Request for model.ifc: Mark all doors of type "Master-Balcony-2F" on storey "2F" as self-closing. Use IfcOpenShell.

First a look at what the model holds.

```python
import ifcopenshell
import ifcopenshell.util.element

model = ifcopenshell.open("model.ifc")
print(model.schema)
storey = next(s for s in model.by_type("IfcBuildingStorey") if s.Name == "2F")
doors = [e for e in ifcopenshell.util.element.get_decomposition(storey) if e.is_a("IfcDoor")]
seen = {}
for e in doors:
    element_type = ifcopenshell.util.element.get_type(e)
    key = (element_type.Name if element_type != e and element_type else None, ifcopenshell.util.element.get_pset(e, "Pset_DoorCommon", "SelfClosing"))
    seen[key] = seen.get(key, 0) + 1
for (name, value), count in sorted(seen.items(), key=str):
    print(count, "x", name, "|", value)
```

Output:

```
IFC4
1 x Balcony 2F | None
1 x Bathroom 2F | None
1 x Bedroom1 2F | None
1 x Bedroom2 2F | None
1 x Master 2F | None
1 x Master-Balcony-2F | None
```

```python
import ifcopenshell
import ifcopenshell.api.pset
import ifcopenshell.util.element

model = ifcopenshell.open("model.ifc")

storey = next(s for s in model.by_type("IfcBuildingStorey") if s.Name == "2F")
doors = [e for e in ifcopenshell.util.element.get_decomposition(storey) if e.is_a("IfcDoor")]

count = 0
for e in doors:
    element_type = ifcopenshell.util.element.get_type(e)
    if element_type in (None, e) or element_type.Name != "Master-Balcony-2F":
        continue
    # add_pset returns the element's existing set when there is one.
    pset = ifcopenshell.api.pset.add_pset(model, product=e, name="Pset_DoorCommon")
    ifcopenshell.api.pset.edit_pset(model, pset=pset, properties={"SelfClosing": True})
    count += 1

print(count, "doors updated")

model.write("model_edited.ifc")
```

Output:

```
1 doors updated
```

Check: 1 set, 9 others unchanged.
